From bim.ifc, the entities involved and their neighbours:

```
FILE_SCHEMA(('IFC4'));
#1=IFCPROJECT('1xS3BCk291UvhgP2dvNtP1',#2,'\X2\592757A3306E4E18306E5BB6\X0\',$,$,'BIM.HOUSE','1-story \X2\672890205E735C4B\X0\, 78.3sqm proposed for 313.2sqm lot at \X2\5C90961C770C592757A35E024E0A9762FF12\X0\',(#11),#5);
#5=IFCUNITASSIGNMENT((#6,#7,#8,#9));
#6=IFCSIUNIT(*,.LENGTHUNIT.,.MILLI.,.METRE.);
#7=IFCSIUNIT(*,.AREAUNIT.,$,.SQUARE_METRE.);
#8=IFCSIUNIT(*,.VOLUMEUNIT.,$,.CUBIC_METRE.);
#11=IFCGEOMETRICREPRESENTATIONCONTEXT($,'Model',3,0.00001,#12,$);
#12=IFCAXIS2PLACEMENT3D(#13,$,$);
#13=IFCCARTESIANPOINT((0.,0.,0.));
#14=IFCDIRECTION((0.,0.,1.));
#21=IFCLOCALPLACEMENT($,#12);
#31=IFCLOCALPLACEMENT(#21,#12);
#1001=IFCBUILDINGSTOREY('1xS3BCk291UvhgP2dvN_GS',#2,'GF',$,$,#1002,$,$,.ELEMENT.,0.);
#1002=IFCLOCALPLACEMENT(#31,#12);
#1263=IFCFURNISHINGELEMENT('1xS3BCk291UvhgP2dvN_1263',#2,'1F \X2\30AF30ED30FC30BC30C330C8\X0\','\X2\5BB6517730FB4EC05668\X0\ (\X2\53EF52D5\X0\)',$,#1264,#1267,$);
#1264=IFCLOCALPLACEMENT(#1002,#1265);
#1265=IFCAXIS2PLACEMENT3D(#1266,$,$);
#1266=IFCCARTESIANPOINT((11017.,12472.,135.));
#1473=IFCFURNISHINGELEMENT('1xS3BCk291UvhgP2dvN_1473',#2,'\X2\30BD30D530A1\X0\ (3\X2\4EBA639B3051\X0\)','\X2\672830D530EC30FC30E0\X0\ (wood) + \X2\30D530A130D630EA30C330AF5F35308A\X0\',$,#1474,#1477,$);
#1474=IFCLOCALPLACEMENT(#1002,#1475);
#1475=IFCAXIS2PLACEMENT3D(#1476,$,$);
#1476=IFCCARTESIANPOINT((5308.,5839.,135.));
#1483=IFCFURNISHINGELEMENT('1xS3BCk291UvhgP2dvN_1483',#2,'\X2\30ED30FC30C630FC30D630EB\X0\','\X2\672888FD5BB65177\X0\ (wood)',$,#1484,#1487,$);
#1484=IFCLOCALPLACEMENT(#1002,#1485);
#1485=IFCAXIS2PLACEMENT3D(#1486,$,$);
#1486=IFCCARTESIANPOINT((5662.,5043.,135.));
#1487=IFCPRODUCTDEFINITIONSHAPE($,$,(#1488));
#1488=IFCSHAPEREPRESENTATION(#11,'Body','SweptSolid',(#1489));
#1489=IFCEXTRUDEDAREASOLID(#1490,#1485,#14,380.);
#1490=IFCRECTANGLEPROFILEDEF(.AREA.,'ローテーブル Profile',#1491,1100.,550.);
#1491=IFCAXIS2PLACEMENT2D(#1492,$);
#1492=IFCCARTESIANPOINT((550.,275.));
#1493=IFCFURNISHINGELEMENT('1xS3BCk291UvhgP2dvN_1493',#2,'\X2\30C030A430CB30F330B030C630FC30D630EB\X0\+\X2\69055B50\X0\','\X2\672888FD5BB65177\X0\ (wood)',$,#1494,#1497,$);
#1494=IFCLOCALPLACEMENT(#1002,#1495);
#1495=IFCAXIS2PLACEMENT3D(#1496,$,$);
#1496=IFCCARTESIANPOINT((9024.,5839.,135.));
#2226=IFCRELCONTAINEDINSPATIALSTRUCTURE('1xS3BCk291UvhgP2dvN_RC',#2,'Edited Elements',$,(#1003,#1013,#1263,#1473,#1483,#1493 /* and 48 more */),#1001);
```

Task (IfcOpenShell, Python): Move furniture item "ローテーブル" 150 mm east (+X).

```python
import ifcopenshell
import ifcopenshell.api.geometry
import ifcopenshell.util.placement
import ifcopenshell.util.unit

model = ifcopenshell.open("bim.ifc")
unit_scale = ifcopenshell.util.unit.calculate_unit_scale(model)

item = model.by_id(1483)
matrix = ifcopenshell.util.placement.get_local_placement(item.ObjectPlacement)
matrix[0, 3] += 0.15 / unit_scale
ifcopenshell.api.geometry.edit_object_placement(model, product=item, matrix=matrix, is_si=False)

print(ifcopenshell.util.placement.get_local_placement(item.ObjectPlacement).round(3) + 0.0)

model.write("bim_v2.ifc")
```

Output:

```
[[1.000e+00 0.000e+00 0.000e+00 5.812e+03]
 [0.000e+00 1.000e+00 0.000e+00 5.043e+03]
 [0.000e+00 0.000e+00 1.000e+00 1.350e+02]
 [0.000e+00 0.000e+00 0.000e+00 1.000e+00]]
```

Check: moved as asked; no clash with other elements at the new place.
